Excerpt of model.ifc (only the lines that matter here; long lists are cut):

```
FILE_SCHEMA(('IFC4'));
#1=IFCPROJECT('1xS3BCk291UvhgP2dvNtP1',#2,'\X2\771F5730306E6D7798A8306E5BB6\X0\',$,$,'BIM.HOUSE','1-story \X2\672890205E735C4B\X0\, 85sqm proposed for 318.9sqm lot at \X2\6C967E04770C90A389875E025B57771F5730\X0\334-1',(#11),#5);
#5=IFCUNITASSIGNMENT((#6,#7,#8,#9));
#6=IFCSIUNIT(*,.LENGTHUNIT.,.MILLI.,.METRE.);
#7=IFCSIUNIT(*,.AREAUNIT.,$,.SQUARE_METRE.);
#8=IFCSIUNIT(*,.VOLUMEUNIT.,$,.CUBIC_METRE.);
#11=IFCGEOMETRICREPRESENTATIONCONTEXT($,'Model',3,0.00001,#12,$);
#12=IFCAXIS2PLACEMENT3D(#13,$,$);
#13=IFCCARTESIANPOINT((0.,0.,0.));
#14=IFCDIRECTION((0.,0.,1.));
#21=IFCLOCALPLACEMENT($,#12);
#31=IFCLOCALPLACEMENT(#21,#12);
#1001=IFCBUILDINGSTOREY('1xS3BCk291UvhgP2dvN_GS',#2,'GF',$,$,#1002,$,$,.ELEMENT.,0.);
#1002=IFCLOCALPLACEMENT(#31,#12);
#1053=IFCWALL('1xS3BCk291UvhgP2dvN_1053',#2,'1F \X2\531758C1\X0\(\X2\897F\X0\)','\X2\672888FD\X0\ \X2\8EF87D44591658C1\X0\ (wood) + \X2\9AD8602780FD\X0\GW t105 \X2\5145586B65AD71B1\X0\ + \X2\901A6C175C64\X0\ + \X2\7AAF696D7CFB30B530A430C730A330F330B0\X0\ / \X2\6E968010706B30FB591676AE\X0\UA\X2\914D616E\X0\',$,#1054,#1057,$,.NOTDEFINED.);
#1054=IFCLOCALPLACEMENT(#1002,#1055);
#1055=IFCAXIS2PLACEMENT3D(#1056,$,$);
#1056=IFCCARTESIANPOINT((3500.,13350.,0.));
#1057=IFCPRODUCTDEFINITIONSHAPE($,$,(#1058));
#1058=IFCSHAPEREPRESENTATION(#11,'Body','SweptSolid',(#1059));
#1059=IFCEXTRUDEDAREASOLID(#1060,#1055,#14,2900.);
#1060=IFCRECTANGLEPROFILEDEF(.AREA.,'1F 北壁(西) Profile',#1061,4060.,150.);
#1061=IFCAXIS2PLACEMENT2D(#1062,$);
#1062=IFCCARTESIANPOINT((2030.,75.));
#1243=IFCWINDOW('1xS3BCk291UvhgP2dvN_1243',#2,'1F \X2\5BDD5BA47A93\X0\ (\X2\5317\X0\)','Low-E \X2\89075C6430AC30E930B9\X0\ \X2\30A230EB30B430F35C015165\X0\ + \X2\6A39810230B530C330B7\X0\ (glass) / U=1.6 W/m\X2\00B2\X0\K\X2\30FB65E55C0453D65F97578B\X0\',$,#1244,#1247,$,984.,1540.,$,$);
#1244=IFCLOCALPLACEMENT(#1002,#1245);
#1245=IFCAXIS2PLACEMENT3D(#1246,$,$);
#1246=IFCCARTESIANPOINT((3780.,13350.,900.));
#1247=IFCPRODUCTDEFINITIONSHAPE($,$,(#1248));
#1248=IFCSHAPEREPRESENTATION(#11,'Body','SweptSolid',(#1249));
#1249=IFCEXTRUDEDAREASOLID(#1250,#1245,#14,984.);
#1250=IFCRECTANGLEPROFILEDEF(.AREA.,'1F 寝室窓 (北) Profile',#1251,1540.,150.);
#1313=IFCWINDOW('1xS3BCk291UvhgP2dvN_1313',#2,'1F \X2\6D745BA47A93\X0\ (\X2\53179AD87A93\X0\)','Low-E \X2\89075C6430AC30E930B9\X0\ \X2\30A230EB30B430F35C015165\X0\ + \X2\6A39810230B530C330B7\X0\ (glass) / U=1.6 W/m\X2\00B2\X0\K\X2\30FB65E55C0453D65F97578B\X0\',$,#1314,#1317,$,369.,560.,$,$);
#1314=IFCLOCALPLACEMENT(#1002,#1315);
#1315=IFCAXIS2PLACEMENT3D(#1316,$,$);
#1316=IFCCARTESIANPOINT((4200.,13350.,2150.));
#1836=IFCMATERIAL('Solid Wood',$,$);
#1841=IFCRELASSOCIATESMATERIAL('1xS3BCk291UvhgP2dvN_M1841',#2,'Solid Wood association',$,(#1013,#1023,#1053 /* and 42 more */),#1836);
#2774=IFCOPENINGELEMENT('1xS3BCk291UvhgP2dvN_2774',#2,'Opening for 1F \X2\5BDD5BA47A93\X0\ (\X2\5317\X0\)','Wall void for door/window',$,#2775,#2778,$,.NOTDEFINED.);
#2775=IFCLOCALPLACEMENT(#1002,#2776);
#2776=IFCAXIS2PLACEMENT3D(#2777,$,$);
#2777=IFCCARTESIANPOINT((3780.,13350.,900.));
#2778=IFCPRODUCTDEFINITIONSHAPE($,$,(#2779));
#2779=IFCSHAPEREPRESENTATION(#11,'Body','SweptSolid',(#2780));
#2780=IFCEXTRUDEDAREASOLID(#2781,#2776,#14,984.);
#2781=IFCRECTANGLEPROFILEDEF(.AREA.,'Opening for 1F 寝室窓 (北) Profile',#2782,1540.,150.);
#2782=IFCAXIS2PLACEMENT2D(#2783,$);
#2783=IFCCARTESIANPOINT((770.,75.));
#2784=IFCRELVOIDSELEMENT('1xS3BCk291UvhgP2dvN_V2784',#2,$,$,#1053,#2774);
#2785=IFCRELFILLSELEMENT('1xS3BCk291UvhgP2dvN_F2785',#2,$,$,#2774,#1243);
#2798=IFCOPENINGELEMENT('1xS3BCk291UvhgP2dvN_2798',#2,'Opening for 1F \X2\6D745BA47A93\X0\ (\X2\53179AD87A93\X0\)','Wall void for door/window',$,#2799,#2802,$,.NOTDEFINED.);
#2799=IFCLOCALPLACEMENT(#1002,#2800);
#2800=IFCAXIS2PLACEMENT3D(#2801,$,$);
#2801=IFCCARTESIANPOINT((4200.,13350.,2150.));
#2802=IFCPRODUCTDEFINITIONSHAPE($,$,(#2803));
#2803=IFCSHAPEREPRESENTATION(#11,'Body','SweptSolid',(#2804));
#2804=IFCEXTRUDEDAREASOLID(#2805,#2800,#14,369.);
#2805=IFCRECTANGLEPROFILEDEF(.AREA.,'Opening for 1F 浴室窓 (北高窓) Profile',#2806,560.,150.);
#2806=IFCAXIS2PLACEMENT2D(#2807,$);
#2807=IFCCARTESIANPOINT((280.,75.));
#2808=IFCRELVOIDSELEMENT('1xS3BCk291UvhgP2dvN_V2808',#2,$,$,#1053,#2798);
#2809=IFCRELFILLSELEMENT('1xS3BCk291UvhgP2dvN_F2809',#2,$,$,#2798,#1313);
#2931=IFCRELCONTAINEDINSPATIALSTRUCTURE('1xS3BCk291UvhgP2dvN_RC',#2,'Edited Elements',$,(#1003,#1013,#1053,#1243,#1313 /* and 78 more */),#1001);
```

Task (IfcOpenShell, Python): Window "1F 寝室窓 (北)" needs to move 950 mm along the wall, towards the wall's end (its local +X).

```python
import ifcopenshell
import ifcopenshell.api.geometry
import ifcopenshell.util.placement
import ifcopenshell.util.unit

model = ifcopenshell.open("model.ifc")
unit_scale = ifcopenshell.util.unit.calculate_unit_scale(model)

window = model.by_guid("1xS3BCk291UvhgP2dvN_1243")
opening = window.FillsVoids[0].RelatingOpeningElement
wall = opening.VoidsElements[0].RelatingBuildingElement

wall_matrix = ifcopenshell.util.placement.get_local_placement(wall.ObjectPlacement)
shift = wall_matrix[:3, 0] * 0.95 / unit_scale
before = ifcopenshell.util.placement.get_local_placement(window.ObjectPlacement)[:3, 3].copy()

# The window is not placed relative to its opening, so move both.
for product in (opening, window):
    matrix = ifcopenshell.util.placement.get_local_placement(product.ObjectPlacement)
    matrix[:3, 3] += shift
    ifcopenshell.api.geometry.edit_object_placement(model, product=product, matrix=matrix, is_si=False)

after = ifcopenshell.util.placement.get_local_placement(window.ObjectPlacement)[:3, 3]
print("window moved by", (after - before).round(3) + 0.0)

model.write("model_updated.ifc")
```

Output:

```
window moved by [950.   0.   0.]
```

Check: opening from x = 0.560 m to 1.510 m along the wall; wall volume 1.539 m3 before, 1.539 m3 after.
